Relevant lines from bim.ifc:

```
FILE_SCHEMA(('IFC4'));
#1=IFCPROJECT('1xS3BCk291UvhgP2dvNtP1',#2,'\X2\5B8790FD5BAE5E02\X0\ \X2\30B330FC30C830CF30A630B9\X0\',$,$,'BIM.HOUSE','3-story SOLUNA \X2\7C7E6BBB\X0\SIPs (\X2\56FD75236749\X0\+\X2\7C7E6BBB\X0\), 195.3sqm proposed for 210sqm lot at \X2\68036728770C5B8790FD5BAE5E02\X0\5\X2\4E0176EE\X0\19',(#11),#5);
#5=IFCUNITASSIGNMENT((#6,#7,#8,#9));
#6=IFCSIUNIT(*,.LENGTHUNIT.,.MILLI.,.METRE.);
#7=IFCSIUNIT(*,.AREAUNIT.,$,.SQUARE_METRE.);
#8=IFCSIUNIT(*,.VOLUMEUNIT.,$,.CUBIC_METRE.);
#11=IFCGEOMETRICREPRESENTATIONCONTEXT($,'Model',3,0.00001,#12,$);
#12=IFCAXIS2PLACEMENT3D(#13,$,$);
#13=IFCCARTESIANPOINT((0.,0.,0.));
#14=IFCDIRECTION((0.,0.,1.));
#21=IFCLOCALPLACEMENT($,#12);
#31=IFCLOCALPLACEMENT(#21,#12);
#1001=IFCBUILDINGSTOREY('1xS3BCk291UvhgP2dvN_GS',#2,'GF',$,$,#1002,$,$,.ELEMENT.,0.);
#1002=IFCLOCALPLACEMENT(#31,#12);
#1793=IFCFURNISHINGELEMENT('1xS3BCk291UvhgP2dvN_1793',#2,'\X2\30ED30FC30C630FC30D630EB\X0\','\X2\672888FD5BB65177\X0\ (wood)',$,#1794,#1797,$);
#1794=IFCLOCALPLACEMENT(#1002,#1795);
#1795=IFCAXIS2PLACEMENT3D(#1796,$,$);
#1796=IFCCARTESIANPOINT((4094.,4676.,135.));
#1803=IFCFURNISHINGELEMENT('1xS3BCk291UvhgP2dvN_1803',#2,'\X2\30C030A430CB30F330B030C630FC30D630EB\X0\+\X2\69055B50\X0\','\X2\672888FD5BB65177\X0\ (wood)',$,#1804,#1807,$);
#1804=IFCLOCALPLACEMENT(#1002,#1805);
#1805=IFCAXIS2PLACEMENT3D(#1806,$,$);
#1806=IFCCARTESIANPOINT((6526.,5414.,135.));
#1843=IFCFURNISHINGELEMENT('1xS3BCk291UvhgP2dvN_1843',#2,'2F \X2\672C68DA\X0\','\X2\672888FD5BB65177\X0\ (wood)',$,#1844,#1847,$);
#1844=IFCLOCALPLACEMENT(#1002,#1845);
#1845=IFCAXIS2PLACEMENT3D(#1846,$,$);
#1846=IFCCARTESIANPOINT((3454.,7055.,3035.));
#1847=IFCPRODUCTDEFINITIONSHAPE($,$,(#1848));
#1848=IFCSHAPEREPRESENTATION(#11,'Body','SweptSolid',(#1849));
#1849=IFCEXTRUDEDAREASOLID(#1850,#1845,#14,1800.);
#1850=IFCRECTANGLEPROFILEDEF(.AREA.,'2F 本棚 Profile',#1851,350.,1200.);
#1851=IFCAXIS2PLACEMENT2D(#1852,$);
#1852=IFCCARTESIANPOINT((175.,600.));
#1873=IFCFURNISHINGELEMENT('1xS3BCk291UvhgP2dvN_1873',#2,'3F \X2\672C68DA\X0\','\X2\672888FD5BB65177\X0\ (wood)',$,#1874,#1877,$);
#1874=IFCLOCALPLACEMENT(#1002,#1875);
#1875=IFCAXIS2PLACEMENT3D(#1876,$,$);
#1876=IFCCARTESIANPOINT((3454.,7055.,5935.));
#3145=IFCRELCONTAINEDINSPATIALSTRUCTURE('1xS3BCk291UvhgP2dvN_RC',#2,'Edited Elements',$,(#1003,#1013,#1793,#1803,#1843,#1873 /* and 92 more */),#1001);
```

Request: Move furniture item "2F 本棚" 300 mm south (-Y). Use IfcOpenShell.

```python
import ifcopenshell
import ifcopenshell.api.geometry
import ifcopenshell.util.placement
import ifcopenshell.util.unit

model = ifcopenshell.open("bim.ifc")
unit_scale = ifcopenshell.util.unit.calculate_unit_scale(model)

item = model.by_guid("1xS3BCk291UvhgP2dvN_1843")
matrix = ifcopenshell.util.placement.get_local_placement(item.ObjectPlacement)
matrix[1, 3] -= 0.3 / unit_scale
ifcopenshell.api.geometry.edit_object_placement(model, product=item, matrix=matrix, is_si=False)

print(ifcopenshell.util.placement.get_local_placement(item.ObjectPlacement).round(3) + 0.0)

model.write("bim_v2.ifc")
```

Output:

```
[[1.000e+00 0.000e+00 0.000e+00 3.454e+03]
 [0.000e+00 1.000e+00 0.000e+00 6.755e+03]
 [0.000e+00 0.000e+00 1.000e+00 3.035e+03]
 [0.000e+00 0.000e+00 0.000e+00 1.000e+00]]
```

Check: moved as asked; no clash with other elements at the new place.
